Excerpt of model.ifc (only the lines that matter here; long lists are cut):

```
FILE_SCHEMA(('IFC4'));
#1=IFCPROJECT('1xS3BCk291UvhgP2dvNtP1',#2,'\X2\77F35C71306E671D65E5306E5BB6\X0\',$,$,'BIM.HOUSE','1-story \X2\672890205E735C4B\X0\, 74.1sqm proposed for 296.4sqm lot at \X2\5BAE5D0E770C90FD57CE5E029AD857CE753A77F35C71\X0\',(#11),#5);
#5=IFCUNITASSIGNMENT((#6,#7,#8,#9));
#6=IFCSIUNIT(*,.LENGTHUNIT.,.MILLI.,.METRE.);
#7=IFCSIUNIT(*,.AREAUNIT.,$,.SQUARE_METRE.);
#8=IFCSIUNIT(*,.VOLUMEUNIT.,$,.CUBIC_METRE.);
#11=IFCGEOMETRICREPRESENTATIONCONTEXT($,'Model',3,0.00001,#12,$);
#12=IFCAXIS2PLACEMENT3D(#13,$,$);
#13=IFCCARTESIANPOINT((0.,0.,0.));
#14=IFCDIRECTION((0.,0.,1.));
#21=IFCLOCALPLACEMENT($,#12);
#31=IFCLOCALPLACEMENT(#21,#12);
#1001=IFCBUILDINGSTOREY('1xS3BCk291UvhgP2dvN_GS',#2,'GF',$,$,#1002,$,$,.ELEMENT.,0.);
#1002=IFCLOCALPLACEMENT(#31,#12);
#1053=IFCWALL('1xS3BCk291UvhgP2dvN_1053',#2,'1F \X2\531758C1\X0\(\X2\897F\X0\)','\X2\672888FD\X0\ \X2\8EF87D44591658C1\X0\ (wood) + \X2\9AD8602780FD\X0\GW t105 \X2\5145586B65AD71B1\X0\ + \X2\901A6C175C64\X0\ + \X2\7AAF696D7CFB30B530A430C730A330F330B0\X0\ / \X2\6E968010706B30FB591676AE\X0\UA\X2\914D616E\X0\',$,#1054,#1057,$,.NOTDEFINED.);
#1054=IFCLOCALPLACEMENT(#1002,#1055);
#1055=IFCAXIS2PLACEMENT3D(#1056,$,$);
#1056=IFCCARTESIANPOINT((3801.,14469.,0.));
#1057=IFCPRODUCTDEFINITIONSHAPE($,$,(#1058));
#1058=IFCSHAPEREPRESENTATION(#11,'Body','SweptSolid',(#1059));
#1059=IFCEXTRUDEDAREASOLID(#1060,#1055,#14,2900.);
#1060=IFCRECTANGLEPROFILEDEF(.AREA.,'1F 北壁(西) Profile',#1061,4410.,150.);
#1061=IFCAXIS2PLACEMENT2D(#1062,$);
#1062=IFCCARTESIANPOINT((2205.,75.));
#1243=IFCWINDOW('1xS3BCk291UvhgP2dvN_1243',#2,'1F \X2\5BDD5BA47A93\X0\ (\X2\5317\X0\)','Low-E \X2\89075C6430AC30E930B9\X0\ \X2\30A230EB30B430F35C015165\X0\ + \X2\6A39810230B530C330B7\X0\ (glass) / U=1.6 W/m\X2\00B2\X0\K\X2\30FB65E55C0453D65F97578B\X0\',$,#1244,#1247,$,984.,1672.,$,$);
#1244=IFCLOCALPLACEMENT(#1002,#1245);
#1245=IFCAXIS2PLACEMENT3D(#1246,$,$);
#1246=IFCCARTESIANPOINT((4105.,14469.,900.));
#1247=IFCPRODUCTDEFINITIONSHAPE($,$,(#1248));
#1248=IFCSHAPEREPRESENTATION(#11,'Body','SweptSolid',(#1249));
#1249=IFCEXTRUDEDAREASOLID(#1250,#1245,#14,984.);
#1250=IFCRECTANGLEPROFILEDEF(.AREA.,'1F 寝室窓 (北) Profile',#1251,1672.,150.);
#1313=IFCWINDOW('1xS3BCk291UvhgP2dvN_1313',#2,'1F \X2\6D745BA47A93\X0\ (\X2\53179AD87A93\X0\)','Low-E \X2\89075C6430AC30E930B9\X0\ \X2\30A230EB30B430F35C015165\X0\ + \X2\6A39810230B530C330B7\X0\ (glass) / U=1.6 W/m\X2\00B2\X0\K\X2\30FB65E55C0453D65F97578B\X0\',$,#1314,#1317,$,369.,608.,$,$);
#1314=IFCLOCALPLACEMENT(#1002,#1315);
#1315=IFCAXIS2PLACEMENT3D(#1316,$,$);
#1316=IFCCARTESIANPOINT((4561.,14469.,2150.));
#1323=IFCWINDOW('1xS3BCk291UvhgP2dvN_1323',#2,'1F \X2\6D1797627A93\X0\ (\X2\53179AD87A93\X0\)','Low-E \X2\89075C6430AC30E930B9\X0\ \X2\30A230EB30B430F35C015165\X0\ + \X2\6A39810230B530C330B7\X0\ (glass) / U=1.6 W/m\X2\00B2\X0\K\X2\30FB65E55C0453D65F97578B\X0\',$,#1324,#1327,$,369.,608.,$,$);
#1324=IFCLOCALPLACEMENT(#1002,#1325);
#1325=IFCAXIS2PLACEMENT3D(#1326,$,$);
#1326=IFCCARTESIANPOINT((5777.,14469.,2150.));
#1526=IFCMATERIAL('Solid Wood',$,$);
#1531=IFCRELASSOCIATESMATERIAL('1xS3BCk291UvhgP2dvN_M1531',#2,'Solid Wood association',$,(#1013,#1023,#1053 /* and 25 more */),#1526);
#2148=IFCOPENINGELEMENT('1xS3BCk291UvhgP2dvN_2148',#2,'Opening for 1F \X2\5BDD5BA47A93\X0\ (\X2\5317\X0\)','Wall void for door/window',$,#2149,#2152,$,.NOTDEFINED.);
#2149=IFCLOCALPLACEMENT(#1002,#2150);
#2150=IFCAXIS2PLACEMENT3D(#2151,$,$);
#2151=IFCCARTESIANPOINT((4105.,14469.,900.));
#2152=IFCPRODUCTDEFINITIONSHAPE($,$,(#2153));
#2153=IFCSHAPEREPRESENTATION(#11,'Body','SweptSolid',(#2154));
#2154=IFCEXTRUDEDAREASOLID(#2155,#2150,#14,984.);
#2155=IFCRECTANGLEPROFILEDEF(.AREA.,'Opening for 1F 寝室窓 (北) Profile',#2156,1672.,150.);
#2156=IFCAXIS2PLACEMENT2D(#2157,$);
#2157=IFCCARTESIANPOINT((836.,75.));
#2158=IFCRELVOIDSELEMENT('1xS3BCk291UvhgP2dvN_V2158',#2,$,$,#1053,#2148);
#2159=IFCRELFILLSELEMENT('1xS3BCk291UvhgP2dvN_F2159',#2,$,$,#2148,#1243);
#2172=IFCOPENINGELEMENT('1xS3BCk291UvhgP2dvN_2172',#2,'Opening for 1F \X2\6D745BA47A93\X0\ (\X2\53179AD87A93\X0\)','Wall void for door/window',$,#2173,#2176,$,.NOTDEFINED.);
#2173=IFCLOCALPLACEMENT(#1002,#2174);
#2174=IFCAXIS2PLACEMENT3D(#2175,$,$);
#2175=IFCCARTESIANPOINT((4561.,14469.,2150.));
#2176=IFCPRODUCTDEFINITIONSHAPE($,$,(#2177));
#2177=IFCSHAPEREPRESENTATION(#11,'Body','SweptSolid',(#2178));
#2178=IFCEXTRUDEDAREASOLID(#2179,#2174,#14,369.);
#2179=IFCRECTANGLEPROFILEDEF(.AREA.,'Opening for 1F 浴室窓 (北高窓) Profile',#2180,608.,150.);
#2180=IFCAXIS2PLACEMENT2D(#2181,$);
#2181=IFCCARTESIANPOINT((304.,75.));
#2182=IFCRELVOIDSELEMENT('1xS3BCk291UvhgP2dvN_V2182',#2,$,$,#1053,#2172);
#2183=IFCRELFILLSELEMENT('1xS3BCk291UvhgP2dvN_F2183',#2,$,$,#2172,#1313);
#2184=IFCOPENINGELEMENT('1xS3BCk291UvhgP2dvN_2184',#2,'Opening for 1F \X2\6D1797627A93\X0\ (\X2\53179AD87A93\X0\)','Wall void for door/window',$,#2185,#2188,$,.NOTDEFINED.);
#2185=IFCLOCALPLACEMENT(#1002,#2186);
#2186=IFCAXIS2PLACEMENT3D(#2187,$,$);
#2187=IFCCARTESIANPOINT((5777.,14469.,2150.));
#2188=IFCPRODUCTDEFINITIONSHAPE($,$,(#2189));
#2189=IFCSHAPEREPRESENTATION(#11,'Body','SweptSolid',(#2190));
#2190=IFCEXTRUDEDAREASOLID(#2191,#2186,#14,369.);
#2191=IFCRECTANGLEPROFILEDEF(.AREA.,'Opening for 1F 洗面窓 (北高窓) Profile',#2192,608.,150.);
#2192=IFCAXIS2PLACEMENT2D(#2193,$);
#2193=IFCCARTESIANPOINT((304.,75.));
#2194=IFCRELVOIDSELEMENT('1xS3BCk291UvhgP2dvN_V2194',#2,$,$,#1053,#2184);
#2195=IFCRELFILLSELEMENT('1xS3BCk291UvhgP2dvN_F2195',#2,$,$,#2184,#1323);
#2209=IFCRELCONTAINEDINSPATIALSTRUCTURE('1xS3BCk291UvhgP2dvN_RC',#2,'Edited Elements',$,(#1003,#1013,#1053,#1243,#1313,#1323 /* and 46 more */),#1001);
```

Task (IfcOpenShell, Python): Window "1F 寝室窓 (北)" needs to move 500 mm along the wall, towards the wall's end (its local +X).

```python
import ifcopenshell
import ifcopenshell.api.geometry
import ifcopenshell.util.placement
import ifcopenshell.util.unit

model = ifcopenshell.open("model.ifc")
unit_scale = ifcopenshell.util.unit.calculate_unit_scale(model)

window = model.by_id(1243)
opening = window.FillsVoids[0].RelatingOpeningElement
wall = opening.VoidsElements[0].RelatingBuildingElement

wall_matrix = ifcopenshell.util.placement.get_local_placement(wall.ObjectPlacement)
shift = wall_matrix[:3, 0] * 0.5 / unit_scale
before = ifcopenshell.util.placement.get_local_placement(window.ObjectPlacement)[:3, 3].copy()

# The window is not placed relative to its opening, so move both.
for product in (opening, window):
    matrix = ifcopenshell.util.placement.get_local_placement(product.ObjectPlacement)
    matrix[:3, 3] += shift
    ifcopenshell.api.geometry.edit_object_placement(model, product=product, matrix=matrix, is_si=False)

after = ifcopenshell.util.placement.get_local_placement(window.ObjectPlacement)[:3, 3]
print("window moved by", (after - before).round(3) + 0.0)

model.write("model_edited.ifc")
```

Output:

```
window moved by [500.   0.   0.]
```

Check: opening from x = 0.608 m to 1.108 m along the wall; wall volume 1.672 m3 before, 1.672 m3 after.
